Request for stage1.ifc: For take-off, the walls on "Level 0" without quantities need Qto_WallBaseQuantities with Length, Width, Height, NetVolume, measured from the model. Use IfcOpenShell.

First a look at what the model holds.

```python
import ifcopenshell
import ifcopenshell.util.element
import ifcopenshell.util.unit

model = ifcopenshell.open("stage1.ifc")
print(model.schema)
for unit_type in ("LENGTHUNIT", "AREAUNIT", "VOLUMEUNIT"):
    print(unit_type, ifcopenshell.util.unit.calculate_unit_scale(model, unit_type))
storey = next(s for s in model.by_type("IfcBuildingStorey") if s.Name == "Level 0")
walls = [e for e in ifcopenshell.util.element.get_decomposition(storey) if e.is_a("IfcWall")]
for e in sorted(walls, key=lambda e: e.id()):
    print(e.id(), e.is_a(), e.Name, list(ifcopenshell.util.element.get_psets(e, qtos_only=True)), sep=" | ")
```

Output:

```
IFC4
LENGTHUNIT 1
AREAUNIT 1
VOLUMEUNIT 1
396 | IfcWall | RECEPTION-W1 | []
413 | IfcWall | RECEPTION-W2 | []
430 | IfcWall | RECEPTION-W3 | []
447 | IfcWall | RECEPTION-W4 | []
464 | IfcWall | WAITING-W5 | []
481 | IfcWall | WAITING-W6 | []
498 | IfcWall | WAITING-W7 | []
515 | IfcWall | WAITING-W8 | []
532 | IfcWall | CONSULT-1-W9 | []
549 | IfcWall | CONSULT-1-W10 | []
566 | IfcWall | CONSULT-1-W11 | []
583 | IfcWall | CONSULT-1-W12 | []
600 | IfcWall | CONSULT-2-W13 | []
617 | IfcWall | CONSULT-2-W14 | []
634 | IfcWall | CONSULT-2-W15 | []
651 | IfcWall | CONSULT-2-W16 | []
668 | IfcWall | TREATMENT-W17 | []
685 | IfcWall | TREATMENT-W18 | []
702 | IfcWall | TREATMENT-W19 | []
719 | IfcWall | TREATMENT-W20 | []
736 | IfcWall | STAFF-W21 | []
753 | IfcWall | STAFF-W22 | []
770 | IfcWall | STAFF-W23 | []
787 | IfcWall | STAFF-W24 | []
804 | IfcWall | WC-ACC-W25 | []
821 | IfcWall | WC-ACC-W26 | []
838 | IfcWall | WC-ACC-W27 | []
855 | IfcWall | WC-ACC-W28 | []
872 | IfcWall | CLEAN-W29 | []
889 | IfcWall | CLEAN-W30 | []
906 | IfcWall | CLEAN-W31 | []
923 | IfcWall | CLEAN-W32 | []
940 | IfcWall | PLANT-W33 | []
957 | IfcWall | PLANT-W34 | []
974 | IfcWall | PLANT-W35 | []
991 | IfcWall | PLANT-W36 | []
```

```python
import ifcopenshell
import ifcopenshell.api.pset
import ifcopenshell.geom
import ifcopenshell.util.element
import ifcopenshell.util.shape
import ifcopenshell.util.unit

model = ifcopenshell.open("stage1.ifc")
unit_scale = ifcopenshell.util.unit.calculate_unit_scale(model)
volume_scale = ifcopenshell.util.unit.calculate_unit_scale(model, "VOLUMEUNIT")
settings = ifcopenshell.geom.settings()

storey = next(s for s in model.by_type("IfcBuildingStorey") if s.Name == "Level 0")
walls = [e for e in ifcopenshell.util.element.get_decomposition(storey) if e.is_a("IfcWall")]

for e in sorted(walls, key=lambda e: e.id()):
    if ifcopenshell.util.element.get_psets(e, qtos_only=True, should_inherit=False):
        continue
    # Geometry comes back in metres, in the element's own axes.
    shape = ifcopenshell.geom.create_shape(settings, e)
    values = {
        "Length": ifcopenshell.util.shape.get_x(shape.geometry) / unit_scale,
        "Width": ifcopenshell.util.shape.get_y(shape.geometry) / unit_scale,
        "Height": ifcopenshell.util.shape.get_z(shape.geometry) / unit_scale,
        "NetVolume": ifcopenshell.util.shape.get_volume(shape.geometry) / volume_scale,
    }
    qto = ifcopenshell.api.pset.add_qto(model, product=e, name="Qto_WallBaseQuantities")
    ifcopenshell.api.pset.edit_qto(model, qto=qto, properties=values)
    print(e.id(), {k: round(v, 3) for k, v in values.items()})

model.write("stage1-out.ifc")
```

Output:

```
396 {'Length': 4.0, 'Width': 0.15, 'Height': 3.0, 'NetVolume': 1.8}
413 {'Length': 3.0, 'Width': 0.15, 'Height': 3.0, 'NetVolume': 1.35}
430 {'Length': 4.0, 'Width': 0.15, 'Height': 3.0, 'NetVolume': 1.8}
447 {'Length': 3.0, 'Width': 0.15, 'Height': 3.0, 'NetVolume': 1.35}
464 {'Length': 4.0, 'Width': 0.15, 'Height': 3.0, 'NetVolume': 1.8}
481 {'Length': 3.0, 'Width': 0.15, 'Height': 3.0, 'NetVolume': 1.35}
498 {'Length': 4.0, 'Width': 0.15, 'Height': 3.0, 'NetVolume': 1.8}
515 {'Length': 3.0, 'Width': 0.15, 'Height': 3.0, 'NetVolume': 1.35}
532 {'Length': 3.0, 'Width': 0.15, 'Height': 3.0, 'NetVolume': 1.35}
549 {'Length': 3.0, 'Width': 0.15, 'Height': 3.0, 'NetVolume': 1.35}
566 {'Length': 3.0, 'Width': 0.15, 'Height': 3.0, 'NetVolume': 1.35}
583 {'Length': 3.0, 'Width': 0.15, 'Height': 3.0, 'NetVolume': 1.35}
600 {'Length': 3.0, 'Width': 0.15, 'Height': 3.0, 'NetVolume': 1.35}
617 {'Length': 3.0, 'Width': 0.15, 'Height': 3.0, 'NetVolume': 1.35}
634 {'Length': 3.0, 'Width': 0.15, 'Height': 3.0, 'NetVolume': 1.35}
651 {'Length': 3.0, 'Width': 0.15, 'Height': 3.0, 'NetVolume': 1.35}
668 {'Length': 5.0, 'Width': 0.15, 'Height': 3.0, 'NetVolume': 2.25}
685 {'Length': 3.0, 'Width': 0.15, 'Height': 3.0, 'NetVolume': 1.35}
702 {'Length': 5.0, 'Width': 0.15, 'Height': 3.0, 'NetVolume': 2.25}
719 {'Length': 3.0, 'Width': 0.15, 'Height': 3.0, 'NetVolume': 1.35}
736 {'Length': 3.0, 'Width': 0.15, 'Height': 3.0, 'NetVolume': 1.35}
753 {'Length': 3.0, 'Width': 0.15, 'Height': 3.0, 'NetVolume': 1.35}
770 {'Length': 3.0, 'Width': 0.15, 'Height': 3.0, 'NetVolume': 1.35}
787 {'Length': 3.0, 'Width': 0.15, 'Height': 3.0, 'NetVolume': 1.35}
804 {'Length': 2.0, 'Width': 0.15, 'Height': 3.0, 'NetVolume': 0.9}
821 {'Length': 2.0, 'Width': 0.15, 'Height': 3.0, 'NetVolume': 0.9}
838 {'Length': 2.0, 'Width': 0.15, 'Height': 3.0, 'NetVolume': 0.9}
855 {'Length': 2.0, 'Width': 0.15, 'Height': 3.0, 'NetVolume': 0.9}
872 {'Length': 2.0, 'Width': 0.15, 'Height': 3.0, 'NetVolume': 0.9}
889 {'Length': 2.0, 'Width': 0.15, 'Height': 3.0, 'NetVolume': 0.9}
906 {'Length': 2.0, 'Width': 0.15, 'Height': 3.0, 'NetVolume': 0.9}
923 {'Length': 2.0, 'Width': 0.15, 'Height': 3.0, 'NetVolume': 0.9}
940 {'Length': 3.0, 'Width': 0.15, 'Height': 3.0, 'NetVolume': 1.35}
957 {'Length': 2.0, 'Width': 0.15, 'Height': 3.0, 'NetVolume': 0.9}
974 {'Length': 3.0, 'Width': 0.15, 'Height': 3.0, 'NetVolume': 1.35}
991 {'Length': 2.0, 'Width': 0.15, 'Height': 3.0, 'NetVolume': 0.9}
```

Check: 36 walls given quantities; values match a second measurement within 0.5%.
